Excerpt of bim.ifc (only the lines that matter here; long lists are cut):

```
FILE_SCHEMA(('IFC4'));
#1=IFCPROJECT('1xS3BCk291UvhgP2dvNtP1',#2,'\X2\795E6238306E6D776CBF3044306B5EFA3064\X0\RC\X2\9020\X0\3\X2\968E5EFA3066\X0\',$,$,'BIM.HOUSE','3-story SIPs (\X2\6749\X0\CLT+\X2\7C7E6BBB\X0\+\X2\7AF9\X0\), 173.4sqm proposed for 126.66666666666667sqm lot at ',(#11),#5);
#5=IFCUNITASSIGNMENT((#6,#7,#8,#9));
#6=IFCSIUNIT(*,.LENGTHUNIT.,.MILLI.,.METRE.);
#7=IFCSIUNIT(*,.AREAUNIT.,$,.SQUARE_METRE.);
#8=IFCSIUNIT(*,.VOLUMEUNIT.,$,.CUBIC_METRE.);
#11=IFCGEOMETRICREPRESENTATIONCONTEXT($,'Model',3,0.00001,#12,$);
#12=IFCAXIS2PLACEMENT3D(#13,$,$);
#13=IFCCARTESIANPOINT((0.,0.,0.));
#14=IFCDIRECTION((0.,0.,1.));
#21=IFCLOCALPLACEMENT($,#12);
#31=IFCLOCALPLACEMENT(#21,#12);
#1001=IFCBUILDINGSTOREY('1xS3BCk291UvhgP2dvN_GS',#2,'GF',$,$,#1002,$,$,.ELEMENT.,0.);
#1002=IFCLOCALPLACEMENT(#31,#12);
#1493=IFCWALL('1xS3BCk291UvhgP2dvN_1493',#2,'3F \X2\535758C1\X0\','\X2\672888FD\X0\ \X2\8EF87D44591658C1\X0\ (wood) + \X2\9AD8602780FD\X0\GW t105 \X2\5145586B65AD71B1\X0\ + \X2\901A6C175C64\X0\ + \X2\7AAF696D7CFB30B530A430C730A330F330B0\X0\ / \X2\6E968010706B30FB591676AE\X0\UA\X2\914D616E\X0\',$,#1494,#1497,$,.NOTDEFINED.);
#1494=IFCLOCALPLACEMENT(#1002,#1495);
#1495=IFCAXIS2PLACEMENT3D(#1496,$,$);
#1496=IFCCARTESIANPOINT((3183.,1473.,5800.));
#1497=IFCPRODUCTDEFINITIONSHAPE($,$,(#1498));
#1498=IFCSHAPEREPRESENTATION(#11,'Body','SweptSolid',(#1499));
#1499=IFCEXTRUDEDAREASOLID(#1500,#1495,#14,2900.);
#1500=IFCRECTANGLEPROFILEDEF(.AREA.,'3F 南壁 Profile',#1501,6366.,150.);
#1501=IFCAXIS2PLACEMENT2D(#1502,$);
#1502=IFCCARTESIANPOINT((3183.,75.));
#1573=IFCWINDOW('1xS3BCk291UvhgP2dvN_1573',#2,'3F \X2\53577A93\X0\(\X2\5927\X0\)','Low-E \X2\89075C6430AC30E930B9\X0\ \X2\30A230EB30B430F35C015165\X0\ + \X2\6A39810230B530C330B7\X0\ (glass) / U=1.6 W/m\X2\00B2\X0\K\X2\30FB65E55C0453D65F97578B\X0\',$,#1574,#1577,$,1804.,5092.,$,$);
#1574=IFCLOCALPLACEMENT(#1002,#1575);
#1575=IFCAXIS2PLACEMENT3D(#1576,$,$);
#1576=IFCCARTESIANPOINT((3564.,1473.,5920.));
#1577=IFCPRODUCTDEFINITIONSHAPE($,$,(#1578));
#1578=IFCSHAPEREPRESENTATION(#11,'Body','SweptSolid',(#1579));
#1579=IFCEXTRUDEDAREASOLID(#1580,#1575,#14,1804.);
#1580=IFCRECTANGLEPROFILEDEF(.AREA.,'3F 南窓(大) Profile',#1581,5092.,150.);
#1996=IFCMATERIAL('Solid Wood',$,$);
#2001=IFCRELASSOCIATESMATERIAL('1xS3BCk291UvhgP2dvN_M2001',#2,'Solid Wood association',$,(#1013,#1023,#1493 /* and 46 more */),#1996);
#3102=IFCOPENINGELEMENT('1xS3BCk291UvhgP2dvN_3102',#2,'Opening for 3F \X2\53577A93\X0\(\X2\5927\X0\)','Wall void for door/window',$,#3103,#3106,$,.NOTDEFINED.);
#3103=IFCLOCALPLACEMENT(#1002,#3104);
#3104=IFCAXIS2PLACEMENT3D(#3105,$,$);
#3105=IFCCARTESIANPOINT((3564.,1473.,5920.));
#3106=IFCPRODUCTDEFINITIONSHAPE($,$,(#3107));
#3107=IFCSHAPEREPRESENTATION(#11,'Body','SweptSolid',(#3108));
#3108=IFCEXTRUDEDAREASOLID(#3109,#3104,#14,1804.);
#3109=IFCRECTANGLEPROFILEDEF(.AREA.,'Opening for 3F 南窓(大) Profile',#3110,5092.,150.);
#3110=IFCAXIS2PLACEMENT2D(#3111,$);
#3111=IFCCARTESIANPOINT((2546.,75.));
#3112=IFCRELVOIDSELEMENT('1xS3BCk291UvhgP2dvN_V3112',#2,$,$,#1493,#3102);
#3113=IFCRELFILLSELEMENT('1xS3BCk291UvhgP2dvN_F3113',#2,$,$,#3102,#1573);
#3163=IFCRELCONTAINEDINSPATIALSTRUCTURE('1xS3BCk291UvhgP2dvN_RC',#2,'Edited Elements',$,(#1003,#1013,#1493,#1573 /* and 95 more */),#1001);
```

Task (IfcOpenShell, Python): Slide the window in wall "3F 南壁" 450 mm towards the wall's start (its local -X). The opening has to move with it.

```python
import ifcopenshell
import ifcopenshell.api.geometry
import ifcopenshell.util.placement

model = ifcopenshell.open("bim.ifc")

window = model.by_guid("1xS3BCk291UvhgP2dvN_1573")
opening = window.FillsVoids[0].RelatingOpeningElement
wall = opening.VoidsElements[0].RelatingBuildingElement

wall_matrix = ifcopenshell.util.placement.get_local_placement(wall.ObjectPlacement)
shift = wall_matrix[:3, 0] * -450.0
before = ifcopenshell.util.placement.get_local_placement(window.ObjectPlacement)[:3, 3].copy()

# The window is not placed relative to its opening, so move both.
for product in (opening, window):
    matrix = ifcopenshell.util.placement.get_local_placement(product.ObjectPlacement)
    matrix[:3, 3] += shift
    ifcopenshell.api.geometry.edit_object_placement(model, product=product, matrix=matrix, is_si=False)

after = ifcopenshell.util.placement.get_local_placement(window.ObjectPlacement)[:3, 3]
print("window moved by", (after - before).round(3) + 0.0)

model.write("bim_edited.ifc")
```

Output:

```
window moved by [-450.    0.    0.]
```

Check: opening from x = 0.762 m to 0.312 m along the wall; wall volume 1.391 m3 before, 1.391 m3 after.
